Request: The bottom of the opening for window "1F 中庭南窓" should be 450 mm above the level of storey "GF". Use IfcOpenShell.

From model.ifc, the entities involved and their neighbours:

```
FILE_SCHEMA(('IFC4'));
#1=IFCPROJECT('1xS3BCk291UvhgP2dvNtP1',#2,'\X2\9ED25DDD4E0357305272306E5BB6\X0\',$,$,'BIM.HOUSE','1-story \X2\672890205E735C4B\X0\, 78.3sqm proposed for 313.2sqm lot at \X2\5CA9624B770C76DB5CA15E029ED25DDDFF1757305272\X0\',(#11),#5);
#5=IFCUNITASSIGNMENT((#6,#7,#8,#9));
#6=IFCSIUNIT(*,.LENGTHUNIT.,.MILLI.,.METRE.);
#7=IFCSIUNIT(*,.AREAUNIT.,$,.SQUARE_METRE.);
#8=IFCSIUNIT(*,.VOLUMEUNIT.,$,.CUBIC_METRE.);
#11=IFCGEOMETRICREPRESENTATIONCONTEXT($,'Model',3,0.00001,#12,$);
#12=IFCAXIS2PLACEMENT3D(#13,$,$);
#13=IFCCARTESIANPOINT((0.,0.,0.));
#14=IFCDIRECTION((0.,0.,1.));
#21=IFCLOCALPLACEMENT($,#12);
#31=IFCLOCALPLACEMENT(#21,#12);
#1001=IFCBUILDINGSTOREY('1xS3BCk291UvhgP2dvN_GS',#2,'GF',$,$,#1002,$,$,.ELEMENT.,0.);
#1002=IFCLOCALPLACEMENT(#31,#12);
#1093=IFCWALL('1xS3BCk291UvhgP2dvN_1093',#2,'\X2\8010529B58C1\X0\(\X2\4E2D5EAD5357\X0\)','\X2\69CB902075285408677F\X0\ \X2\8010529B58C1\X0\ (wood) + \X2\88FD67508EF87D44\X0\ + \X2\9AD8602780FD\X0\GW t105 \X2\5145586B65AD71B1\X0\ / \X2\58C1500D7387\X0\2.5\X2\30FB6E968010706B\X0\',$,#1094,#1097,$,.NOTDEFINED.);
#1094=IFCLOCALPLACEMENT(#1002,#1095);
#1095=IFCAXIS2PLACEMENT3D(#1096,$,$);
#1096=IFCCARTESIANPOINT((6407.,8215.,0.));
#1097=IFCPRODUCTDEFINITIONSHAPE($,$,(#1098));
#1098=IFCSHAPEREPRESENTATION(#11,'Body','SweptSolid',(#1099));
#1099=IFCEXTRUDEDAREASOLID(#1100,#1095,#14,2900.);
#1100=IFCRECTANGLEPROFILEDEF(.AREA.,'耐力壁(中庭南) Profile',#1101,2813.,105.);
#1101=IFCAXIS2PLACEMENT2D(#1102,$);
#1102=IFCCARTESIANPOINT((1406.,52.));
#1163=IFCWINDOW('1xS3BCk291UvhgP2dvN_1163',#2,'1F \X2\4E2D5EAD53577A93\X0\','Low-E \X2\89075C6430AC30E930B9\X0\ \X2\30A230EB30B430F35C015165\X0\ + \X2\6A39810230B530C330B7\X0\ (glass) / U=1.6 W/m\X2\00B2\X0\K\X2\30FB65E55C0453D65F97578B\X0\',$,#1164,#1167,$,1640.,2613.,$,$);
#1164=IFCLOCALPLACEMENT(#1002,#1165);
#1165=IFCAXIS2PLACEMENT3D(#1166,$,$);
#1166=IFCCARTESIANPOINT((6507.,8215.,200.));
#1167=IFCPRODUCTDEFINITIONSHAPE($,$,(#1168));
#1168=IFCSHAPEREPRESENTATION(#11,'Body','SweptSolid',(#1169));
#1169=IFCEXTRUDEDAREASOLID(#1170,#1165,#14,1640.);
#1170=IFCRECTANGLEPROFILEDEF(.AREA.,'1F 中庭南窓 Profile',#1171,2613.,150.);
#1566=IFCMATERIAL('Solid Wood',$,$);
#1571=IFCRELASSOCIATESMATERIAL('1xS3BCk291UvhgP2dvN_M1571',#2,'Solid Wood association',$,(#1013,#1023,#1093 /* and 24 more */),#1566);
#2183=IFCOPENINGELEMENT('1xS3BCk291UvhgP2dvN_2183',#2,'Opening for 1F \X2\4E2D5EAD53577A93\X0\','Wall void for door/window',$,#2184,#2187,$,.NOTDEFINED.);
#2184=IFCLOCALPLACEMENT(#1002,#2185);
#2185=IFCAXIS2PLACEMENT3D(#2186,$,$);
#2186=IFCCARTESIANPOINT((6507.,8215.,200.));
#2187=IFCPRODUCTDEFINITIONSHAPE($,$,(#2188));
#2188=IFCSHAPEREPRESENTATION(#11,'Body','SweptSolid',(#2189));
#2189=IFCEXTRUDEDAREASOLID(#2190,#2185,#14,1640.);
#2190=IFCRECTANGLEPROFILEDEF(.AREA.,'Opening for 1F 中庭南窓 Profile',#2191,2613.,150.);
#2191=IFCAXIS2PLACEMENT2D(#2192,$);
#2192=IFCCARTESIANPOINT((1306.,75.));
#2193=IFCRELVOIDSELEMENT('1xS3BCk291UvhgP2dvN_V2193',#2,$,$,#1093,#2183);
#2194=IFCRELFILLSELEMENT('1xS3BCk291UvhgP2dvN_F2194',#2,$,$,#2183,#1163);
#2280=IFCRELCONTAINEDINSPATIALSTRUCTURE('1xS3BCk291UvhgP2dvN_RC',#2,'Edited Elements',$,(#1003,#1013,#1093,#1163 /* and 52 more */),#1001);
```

```python
import numpy as np
import ifcopenshell
import ifcopenshell.api.geometry
import ifcopenshell.geom
import ifcopenshell.util.element
import ifcopenshell.util.placement
import ifcopenshell.util.shape
import ifcopenshell.util.unit

model = ifcopenshell.open("model.ifc")
unit_scale = ifcopenshell.util.unit.calculate_unit_scale(model)

window = model.by_id(1163)
opening = window.FillsVoids[0].RelatingOpeningElement
storey = ifcopenshell.util.element.get_container(window, ifc_class="IfcBuildingStorey")
level = ifcopenshell.util.placement.get_local_placement(storey.ObjectPlacement)[2, 3]

# The opening's origin need not be at the sill, so measure its lowest point.
shape = ifcopenshell.geom.create_shape(ifcopenshell.geom.settings(), opening)
bottom = ifcopenshell.util.shape.get_shape_bottom_elevation(shape, shape.geometry) / unit_scale
dz = level + 0.45 / unit_scale - bottom

shift = np.array([0.0, 0.0, dz])
# The window is not placed relative to its opening, so move both.
for product in (opening, window):
    matrix = ifcopenshell.util.placement.get_local_placement(product.ObjectPlacement)
    matrix[:3, 3] += shift
    ifcopenshell.api.geometry.edit_object_placement(model, product=product, matrix=matrix, is_si=False)

print(f"moved by {dz * unit_scale:+.3f} m")

model.write("model_rev.ifc")
```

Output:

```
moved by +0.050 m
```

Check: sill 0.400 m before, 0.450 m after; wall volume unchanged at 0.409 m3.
